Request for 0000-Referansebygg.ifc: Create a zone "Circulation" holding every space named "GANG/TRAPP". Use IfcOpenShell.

First a look at what the model holds.

```python
import ifcopenshell

model = ifcopenshell.open("0000-Referansebygg.ifc")
print(model.schema)
seen = {}
for space in model.by_type("IfcSpace"):
    seen[space.LongName] = seen.get(space.LongName, 0) + 1
for name, count in sorted(seen.items(), key=str):
    print(count, "x", name)
print("zones:", [z.Name for z in model.by_type("IfcZone")][:20])
```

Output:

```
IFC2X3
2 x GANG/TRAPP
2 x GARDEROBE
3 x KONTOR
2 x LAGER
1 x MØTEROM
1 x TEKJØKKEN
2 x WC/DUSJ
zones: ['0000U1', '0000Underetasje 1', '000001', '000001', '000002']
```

```python
import ifcopenshell
import ifcopenshell.api.group
import ifcopenshell.api.root

model = ifcopenshell.open("0000-Referansebygg.ifc")

names = {"GANG/TRAPP"}
spaces = [s for s in model.by_type("IfcSpace") if s.LongName in names]

zone = ifcopenshell.api.root.create_entity(model, ifc_class="IfcZone", name="Circulation")
ifcopenshell.api.group.assign_group(model, products=spaces, group=zone)
print(len(spaces), "spaces in", zone.Name)

model.write("0000-Referansebygg_rev.ifc")
```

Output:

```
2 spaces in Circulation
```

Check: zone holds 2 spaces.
